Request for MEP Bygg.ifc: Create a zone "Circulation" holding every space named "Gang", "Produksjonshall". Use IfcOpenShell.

First a look at what the model holds.

```python
import ifcopenshell

model = ifcopenshell.open("MEP Bygg.ifc")
print(model.schema)
seen = {}
for space in model.by_type("IfcSpace"):
    seen[space.LongName] = seen.get(space.LongName, 0) + 1
for name, count in sorted(seen.items(), key=str):
    print(count, "x", name)
print("zones:", [z.Name for z in model.by_type("IfcZone")][:20])
```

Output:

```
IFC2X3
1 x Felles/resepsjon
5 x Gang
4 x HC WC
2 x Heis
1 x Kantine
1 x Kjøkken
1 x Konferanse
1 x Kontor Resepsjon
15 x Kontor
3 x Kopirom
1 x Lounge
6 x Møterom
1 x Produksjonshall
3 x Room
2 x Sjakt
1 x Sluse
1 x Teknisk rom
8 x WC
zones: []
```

```python
import ifcopenshell
import ifcopenshell.api.group
import ifcopenshell.api.root

model = ifcopenshell.open("MEP Bygg.ifc")

names = {"Gang", "Produksjonshall"}
spaces = [s for s in model.by_type("IfcSpace") if s.LongName in names]

zone = ifcopenshell.api.root.create_entity(model, ifc_class="IfcZone", name="Circulation")
ifcopenshell.api.group.assign_group(model, products=spaces, group=zone)
print(len(spaces), "spaces in", zone.Name)

model.write("MEP Bygg_v2.ifc")
```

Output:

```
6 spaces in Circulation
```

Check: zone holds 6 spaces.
